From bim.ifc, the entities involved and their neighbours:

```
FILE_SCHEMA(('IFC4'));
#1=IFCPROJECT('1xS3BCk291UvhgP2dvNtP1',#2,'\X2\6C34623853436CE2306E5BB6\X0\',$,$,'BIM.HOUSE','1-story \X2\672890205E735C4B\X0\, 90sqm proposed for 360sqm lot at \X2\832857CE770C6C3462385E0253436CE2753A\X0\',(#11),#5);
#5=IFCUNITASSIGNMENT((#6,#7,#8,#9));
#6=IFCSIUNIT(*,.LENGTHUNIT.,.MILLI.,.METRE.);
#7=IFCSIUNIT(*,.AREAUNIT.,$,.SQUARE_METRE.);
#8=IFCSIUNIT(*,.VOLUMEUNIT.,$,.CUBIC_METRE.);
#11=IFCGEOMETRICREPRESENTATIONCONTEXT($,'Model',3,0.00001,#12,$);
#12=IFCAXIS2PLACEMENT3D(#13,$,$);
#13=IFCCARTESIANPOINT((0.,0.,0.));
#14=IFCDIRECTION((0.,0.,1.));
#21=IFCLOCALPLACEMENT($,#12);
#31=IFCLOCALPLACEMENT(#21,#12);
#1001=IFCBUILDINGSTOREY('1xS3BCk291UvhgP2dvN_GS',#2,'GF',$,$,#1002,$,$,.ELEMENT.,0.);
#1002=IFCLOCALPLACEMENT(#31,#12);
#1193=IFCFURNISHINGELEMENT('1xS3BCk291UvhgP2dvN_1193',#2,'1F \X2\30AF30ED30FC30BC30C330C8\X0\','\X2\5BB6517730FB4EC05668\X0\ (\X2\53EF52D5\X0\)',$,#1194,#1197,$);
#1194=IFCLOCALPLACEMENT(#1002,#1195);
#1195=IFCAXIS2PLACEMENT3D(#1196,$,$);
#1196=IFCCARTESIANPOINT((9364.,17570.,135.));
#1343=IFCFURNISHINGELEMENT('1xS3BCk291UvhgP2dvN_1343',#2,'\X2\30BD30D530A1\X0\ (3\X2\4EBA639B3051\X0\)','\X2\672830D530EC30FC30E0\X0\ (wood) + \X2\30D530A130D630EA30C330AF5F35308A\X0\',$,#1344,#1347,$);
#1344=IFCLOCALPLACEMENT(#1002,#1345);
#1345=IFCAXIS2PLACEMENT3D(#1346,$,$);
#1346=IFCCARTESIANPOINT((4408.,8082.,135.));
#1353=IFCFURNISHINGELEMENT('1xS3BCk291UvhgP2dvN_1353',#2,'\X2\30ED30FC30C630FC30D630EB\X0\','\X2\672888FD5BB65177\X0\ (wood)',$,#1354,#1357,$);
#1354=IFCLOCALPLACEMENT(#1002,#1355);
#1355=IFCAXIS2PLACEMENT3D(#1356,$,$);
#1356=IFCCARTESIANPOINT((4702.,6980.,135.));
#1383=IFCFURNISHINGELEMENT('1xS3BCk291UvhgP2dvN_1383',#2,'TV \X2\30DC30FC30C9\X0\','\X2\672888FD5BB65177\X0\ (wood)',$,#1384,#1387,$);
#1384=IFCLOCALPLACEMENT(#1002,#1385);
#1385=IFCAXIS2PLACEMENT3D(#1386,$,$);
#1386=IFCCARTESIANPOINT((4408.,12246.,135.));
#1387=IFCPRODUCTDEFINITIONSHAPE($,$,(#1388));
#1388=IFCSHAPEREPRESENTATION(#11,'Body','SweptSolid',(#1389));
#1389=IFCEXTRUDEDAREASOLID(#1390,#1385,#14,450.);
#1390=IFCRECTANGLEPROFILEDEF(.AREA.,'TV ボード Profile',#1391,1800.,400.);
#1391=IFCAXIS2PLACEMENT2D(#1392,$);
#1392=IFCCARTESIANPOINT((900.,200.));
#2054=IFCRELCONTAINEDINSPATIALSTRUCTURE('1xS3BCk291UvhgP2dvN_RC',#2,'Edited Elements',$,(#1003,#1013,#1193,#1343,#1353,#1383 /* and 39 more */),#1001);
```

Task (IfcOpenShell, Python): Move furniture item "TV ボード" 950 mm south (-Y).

```python
import ifcopenshell
import ifcopenshell.api.geometry
import ifcopenshell.util.placement
import ifcopenshell.util.unit

model = ifcopenshell.open("bim.ifc")
unit_scale = ifcopenshell.util.unit.calculate_unit_scale(model)

item = model.by_id(1383)
matrix = ifcopenshell.util.placement.get_local_placement(item.ObjectPlacement)
matrix[1, 3] -= 0.95 / unit_scale
ifcopenshell.api.geometry.edit_object_placement(model, product=item, matrix=matrix, is_si=False)

print(ifcopenshell.util.placement.get_local_placement(item.ObjectPlacement).round(3) + 0.0)

model.write("bim_v2.ifc")
```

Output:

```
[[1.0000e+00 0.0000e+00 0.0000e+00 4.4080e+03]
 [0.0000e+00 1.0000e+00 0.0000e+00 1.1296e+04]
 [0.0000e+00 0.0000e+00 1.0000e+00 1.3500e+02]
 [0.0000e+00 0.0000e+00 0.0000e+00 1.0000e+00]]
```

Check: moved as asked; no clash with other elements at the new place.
